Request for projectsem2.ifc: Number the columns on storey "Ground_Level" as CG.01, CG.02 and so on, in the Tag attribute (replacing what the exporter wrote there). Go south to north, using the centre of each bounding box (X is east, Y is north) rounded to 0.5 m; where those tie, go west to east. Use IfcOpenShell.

First a look at what the model holds.

```python
import ifcopenshell
import ifcopenshell.util.element
import ifcopenshell.util.placement

model = ifcopenshell.open("projectsem2.ifc")
print(model.schema)
storey = next(s for s in model.by_type("IfcBuildingStorey") if s.Name == "Ground_Level")
columns = [e for e in ifcopenshell.util.element.get_decomposition(storey) if e.is_a("IfcColumn")]
for e in sorted(columns, key=lambda e: e.id()):
    origin = ifcopenshell.util.placement.get_local_placement(e.ObjectPlacement)[:3, 3]
    print(e.id(), e.Tag, e.Name, origin.round(2) + 0.0, sep=" | ")
```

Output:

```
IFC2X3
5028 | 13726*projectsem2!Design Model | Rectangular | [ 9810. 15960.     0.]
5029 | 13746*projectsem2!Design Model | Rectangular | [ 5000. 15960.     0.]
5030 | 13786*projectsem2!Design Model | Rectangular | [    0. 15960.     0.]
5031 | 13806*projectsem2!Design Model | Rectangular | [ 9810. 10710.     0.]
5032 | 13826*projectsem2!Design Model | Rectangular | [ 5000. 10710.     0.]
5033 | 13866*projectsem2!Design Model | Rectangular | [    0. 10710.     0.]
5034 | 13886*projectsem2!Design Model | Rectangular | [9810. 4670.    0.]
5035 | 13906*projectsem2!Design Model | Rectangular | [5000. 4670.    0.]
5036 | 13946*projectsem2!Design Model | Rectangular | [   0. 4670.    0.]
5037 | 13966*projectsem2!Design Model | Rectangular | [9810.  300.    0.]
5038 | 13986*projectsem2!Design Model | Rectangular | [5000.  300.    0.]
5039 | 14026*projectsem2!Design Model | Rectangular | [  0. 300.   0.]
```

```python
import ifcopenshell
import ifcopenshell.geom
import ifcopenshell.util.element
import ifcopenshell.util.shape

model = ifcopenshell.open("projectsem2.ifc")
settings = ifcopenshell.geom.settings()
settings.set("use-world-coords", True)


def centre(element):
    shape = ifcopenshell.geom.create_shape(settings, element)
    return ifcopenshell.util.shape.get_bbox_centroid(shape.geometry)


storey = next(s for s in model.by_type("IfcBuildingStorey") if s.Name == "Ground_Level")
columns = [e for e in ifcopenshell.util.element.get_decomposition(storey) if e.is_a("IfcColumn")]

# Insertion points can sit at a corner or the storey origin, so sort by the geometry (in metres).
centres = {e: centre(e) for e in columns}
columns.sort(key=lambda e: (round(centres[e][1] / 0.5), centres[e][0]))

for i, e in enumerate(columns, start=1):
    number = f"CG.{i:02d}"
    e.Tag = number
    print(e.id(), number)

model.write("projectsem2-out.ifc")
```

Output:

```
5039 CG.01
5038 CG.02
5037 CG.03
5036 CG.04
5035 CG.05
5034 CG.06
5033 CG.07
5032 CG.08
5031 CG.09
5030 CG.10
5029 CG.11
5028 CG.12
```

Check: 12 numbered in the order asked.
